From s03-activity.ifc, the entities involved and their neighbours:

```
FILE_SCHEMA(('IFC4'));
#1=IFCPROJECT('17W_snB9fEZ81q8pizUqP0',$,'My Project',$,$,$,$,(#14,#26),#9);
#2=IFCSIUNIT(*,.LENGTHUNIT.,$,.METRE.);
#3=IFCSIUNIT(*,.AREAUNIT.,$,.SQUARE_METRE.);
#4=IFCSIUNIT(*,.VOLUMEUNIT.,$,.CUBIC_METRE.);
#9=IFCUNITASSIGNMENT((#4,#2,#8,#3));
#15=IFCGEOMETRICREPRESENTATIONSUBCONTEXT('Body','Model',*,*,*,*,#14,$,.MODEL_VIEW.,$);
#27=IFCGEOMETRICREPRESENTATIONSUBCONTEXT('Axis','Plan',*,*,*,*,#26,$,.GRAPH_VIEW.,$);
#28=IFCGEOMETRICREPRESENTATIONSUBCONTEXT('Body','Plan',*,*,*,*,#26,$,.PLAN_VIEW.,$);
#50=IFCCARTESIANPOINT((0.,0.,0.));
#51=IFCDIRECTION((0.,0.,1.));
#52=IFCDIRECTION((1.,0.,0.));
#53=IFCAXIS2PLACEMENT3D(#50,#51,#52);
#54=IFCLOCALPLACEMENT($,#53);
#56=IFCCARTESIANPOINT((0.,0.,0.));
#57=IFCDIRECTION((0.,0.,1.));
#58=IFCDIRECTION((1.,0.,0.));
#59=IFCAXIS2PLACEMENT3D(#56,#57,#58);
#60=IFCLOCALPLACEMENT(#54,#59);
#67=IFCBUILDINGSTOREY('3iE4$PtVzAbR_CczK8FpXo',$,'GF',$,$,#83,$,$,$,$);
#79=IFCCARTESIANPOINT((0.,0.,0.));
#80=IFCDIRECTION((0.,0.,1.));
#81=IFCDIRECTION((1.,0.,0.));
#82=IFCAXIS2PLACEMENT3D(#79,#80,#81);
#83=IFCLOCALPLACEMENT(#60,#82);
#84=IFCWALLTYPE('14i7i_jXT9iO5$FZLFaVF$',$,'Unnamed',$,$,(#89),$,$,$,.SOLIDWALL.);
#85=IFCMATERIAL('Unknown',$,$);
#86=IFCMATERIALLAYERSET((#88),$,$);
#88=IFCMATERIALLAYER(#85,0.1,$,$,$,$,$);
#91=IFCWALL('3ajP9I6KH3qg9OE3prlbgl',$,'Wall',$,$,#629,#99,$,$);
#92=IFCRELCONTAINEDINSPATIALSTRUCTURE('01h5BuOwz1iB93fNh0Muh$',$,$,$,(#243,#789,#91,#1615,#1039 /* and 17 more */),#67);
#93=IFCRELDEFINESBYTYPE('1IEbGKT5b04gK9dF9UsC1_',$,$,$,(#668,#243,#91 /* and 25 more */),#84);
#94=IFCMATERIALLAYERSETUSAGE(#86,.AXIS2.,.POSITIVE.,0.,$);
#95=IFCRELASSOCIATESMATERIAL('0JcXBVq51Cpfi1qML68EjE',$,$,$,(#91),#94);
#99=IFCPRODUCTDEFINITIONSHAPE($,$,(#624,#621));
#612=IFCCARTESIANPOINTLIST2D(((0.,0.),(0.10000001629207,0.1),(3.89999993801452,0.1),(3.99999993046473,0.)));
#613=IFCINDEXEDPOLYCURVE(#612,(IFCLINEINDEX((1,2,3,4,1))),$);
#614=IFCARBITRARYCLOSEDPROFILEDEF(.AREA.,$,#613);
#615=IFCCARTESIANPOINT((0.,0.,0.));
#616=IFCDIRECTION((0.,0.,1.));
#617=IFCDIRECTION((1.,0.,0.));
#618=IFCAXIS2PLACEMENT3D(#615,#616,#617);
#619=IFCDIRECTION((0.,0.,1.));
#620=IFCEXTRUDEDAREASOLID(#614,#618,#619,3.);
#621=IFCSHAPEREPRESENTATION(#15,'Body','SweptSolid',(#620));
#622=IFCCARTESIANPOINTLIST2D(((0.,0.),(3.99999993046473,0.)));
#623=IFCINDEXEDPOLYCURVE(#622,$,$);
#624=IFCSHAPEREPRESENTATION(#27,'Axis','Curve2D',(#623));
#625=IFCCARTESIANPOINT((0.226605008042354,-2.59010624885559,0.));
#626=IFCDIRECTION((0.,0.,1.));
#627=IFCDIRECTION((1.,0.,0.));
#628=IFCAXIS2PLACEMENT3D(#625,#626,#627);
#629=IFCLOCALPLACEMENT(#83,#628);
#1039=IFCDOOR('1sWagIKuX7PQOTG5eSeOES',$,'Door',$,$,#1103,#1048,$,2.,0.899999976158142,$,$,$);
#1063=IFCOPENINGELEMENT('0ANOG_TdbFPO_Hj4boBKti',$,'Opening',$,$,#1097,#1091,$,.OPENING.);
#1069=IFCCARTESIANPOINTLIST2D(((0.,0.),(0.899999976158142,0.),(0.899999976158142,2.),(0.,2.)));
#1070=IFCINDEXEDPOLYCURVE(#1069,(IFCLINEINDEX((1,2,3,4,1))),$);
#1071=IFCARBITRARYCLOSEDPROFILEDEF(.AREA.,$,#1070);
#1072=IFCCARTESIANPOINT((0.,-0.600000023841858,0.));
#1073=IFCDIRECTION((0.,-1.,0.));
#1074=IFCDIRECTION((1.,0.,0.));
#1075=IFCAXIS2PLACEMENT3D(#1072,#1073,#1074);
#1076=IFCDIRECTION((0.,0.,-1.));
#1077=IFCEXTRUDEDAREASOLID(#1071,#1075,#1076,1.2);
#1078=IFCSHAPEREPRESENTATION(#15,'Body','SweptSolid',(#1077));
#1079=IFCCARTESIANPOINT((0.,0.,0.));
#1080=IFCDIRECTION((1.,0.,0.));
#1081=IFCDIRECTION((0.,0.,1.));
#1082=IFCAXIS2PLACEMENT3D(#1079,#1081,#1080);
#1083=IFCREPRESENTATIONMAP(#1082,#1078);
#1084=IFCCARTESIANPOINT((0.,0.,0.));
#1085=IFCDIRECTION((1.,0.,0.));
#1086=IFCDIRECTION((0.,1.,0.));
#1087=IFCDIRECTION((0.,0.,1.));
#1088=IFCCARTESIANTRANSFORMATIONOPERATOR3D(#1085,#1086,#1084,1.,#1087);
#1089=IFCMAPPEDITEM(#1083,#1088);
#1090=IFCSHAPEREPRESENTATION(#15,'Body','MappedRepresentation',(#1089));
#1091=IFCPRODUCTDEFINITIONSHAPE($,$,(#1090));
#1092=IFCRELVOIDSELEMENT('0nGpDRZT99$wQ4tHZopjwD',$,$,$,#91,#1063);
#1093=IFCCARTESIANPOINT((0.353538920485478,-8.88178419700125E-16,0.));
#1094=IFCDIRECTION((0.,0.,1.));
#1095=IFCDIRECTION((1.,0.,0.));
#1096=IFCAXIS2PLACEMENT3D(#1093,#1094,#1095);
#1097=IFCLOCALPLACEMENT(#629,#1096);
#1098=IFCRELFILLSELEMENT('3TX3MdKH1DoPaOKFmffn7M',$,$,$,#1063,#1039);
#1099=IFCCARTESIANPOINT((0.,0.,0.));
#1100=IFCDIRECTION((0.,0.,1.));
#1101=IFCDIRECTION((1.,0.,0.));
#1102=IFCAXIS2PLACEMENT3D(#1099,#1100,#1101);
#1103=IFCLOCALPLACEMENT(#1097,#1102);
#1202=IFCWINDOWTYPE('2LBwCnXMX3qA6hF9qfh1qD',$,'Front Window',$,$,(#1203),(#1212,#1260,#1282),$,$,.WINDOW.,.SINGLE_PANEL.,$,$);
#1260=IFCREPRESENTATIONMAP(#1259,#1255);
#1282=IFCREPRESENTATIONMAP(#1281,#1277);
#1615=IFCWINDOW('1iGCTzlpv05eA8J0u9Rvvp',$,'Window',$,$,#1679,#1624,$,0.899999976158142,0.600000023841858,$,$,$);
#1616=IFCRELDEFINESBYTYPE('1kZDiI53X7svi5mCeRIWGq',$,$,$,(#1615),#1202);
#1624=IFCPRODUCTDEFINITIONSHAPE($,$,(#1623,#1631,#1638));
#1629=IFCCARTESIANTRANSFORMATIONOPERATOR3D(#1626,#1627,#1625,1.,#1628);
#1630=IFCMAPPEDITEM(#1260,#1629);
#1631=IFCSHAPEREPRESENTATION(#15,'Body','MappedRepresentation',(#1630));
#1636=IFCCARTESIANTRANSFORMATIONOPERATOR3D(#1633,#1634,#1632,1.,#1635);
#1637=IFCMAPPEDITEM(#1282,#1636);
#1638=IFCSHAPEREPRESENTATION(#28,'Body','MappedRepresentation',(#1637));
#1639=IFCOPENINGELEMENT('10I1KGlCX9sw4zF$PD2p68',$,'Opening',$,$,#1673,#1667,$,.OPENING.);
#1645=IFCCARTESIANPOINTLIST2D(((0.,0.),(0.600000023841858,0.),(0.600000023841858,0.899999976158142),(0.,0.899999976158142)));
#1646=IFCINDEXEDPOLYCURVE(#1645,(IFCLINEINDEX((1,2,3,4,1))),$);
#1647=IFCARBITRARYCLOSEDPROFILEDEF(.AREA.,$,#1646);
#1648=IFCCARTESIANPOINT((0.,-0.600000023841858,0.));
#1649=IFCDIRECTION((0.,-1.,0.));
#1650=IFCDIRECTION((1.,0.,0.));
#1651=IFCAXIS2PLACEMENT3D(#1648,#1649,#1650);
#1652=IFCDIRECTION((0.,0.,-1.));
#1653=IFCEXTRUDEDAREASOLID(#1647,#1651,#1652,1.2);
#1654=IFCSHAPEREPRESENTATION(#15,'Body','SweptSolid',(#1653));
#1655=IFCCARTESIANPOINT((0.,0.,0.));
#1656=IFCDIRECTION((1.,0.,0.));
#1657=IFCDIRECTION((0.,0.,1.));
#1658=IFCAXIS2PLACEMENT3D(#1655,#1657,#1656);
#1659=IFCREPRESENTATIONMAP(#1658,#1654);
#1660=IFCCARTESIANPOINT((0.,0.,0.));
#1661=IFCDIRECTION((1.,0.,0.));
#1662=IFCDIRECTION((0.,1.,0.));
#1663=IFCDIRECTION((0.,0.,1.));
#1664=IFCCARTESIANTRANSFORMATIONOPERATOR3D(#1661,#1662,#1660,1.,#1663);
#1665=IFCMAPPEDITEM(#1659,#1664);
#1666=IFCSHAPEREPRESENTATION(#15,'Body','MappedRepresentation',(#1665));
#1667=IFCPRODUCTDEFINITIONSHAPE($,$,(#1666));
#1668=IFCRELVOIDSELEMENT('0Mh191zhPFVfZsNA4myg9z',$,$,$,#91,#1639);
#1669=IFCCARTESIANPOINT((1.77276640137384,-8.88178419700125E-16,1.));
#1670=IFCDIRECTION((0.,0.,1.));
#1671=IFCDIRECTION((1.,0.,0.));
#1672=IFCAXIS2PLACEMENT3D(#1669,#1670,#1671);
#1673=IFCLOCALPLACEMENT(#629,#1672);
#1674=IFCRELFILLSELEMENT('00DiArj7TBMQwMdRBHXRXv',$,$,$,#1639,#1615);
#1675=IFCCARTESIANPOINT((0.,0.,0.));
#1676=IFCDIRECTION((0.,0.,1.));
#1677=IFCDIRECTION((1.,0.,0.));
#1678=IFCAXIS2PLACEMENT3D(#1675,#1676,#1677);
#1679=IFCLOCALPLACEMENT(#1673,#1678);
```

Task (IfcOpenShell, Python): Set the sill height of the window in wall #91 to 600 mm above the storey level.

```python
import numpy as np
import ifcopenshell
import ifcopenshell.api.geometry
import ifcopenshell.geom
import ifcopenshell.util.element
import ifcopenshell.util.placement
import ifcopenshell.util.shape
import ifcopenshell.util.unit

model = ifcopenshell.open("s03-activity.ifc")
unit_scale = ifcopenshell.util.unit.calculate_unit_scale(model)

window = model.by_guid("1iGCTzlpv05eA8J0u9Rvvp")
opening = window.FillsVoids[0].RelatingOpeningElement
storey = ifcopenshell.util.element.get_container(window, ifc_class="IfcBuildingStorey")
level = ifcopenshell.util.placement.get_local_placement(storey.ObjectPlacement)[2, 3]

# The opening's origin need not be at the sill, so measure its lowest point.
shape = ifcopenshell.geom.create_shape(ifcopenshell.geom.settings(), opening)
bottom = ifcopenshell.util.shape.get_shape_bottom_elevation(shape, shape.geometry) / unit_scale
dz = level + 0.6 / unit_scale - bottom

shift = np.array([0.0, 0.0, dz])
# The window is placed relative to its opening, so it follows when the opening moves.
matrix = ifcopenshell.util.placement.get_local_placement(opening.ObjectPlacement)
matrix[:3, 3] += shift
ifcopenshell.api.geometry.edit_object_placement(
    model, product=opening, matrix=matrix, is_si=False, should_transform_children=True
)

print(f"moved by {dz * unit_scale:+.3f} m")

model.write("s03-activity_updated.ifc")
```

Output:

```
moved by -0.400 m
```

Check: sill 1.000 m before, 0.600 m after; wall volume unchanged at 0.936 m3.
